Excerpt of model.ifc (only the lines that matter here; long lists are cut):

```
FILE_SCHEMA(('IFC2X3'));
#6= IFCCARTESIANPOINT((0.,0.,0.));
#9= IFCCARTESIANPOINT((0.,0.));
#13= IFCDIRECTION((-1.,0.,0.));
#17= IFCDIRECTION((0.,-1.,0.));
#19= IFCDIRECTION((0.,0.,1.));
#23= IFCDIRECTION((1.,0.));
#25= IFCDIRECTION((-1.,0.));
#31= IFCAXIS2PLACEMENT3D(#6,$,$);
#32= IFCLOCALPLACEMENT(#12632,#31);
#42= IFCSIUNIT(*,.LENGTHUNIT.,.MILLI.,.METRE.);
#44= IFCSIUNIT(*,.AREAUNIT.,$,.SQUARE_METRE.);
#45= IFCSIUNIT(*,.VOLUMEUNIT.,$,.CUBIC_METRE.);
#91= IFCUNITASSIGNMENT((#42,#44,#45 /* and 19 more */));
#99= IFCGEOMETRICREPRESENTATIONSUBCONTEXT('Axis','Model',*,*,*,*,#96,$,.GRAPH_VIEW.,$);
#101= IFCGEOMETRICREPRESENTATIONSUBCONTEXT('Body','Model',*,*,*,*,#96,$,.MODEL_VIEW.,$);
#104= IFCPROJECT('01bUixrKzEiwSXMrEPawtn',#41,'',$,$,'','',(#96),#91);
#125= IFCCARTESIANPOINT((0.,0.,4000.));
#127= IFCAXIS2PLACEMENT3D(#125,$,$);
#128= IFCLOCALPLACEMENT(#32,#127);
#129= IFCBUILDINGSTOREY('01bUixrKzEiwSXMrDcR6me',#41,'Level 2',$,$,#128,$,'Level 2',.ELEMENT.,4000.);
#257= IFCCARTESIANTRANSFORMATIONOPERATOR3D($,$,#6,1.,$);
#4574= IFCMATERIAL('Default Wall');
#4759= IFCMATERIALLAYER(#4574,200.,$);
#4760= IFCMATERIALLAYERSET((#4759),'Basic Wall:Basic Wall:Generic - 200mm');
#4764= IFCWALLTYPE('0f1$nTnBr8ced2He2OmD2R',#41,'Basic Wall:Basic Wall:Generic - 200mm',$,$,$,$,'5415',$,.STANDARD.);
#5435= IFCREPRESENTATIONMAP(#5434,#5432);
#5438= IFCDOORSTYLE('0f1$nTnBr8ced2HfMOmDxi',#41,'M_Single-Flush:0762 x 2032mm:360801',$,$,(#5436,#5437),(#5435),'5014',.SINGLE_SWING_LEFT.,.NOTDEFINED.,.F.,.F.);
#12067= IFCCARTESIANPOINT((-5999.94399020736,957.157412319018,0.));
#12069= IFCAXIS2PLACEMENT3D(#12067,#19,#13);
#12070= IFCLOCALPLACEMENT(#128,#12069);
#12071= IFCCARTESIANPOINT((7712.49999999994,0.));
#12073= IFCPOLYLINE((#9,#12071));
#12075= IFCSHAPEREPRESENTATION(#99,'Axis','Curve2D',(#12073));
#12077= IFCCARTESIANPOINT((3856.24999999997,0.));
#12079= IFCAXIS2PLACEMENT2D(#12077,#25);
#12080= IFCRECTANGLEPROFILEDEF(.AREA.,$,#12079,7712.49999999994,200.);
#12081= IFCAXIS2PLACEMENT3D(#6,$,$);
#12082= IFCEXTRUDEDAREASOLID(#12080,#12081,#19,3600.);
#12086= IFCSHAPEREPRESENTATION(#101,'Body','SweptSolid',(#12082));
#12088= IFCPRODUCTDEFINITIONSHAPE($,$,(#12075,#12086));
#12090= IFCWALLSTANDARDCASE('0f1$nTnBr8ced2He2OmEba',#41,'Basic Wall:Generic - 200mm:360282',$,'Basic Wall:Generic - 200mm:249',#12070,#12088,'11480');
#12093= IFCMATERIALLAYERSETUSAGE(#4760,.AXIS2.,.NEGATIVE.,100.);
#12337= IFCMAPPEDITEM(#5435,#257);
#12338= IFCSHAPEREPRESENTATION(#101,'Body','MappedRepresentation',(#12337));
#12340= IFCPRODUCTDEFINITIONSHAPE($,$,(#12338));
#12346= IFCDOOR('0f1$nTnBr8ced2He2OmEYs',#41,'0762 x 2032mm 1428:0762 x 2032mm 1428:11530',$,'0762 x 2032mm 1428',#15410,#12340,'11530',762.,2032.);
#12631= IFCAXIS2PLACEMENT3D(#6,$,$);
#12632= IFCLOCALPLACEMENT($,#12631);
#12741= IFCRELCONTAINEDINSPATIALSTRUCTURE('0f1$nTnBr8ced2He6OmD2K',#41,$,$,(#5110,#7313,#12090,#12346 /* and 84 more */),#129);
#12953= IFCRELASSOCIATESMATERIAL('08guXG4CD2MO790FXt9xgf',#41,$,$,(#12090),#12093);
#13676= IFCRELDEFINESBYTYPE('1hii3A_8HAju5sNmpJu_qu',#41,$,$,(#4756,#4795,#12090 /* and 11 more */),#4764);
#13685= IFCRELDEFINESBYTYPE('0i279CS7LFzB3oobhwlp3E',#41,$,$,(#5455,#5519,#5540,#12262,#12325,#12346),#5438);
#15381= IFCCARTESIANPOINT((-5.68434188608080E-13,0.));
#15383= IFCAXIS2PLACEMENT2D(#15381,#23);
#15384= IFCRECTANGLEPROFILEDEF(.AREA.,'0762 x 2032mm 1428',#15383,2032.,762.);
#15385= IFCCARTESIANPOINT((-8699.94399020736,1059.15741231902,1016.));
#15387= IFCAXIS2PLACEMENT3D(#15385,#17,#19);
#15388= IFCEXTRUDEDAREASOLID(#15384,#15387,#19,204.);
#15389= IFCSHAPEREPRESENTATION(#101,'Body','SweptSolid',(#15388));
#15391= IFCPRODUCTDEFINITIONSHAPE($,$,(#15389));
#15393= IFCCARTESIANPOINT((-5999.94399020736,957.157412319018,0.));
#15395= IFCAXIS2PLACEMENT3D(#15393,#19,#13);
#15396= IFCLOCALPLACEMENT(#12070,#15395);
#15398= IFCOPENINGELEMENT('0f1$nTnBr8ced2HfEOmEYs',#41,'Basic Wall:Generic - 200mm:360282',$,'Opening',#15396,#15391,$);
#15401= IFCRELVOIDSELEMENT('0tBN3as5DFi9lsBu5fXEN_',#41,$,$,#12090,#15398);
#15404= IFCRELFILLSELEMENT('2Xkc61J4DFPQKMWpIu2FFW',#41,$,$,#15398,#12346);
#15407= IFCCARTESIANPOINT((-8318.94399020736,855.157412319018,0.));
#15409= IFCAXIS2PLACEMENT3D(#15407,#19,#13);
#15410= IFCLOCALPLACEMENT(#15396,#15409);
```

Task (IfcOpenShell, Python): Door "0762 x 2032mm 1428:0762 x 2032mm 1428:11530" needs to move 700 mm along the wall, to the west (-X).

```python
import ifcopenshell
import ifcopenshell.api.geometry
import ifcopenshell.util.placement

model = ifcopenshell.open("model.ifc")

door = model.by_guid("0f1$nTnBr8ced2He2OmEYs")
opening = door.FillsVoids[0].RelatingOpeningElement
wall = opening.VoidsElements[0].RelatingBuildingElement

wall_matrix = ifcopenshell.util.placement.get_local_placement(wall.ObjectPlacement)
shift = wall_matrix[:3, 0] * 700.0
before = ifcopenshell.util.placement.get_local_placement(door.ObjectPlacement)[:3, 3].copy()

# The door is placed relative to its opening, so it follows when the opening moves.
matrix = ifcopenshell.util.placement.get_local_placement(opening.ObjectPlacement)
matrix[:3, 3] += shift
ifcopenshell.api.geometry.edit_object_placement(
    model, product=opening, matrix=matrix, is_si=False, should_transform_children=True
)

after = ifcopenshell.util.placement.get_local_placement(door.ObjectPlacement)[:3, 3]
print("door moved by", (after - before).round(3) + 0.0)

model.write("model_edited.ifc")
```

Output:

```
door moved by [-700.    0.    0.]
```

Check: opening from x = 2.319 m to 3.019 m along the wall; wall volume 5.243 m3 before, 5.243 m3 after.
